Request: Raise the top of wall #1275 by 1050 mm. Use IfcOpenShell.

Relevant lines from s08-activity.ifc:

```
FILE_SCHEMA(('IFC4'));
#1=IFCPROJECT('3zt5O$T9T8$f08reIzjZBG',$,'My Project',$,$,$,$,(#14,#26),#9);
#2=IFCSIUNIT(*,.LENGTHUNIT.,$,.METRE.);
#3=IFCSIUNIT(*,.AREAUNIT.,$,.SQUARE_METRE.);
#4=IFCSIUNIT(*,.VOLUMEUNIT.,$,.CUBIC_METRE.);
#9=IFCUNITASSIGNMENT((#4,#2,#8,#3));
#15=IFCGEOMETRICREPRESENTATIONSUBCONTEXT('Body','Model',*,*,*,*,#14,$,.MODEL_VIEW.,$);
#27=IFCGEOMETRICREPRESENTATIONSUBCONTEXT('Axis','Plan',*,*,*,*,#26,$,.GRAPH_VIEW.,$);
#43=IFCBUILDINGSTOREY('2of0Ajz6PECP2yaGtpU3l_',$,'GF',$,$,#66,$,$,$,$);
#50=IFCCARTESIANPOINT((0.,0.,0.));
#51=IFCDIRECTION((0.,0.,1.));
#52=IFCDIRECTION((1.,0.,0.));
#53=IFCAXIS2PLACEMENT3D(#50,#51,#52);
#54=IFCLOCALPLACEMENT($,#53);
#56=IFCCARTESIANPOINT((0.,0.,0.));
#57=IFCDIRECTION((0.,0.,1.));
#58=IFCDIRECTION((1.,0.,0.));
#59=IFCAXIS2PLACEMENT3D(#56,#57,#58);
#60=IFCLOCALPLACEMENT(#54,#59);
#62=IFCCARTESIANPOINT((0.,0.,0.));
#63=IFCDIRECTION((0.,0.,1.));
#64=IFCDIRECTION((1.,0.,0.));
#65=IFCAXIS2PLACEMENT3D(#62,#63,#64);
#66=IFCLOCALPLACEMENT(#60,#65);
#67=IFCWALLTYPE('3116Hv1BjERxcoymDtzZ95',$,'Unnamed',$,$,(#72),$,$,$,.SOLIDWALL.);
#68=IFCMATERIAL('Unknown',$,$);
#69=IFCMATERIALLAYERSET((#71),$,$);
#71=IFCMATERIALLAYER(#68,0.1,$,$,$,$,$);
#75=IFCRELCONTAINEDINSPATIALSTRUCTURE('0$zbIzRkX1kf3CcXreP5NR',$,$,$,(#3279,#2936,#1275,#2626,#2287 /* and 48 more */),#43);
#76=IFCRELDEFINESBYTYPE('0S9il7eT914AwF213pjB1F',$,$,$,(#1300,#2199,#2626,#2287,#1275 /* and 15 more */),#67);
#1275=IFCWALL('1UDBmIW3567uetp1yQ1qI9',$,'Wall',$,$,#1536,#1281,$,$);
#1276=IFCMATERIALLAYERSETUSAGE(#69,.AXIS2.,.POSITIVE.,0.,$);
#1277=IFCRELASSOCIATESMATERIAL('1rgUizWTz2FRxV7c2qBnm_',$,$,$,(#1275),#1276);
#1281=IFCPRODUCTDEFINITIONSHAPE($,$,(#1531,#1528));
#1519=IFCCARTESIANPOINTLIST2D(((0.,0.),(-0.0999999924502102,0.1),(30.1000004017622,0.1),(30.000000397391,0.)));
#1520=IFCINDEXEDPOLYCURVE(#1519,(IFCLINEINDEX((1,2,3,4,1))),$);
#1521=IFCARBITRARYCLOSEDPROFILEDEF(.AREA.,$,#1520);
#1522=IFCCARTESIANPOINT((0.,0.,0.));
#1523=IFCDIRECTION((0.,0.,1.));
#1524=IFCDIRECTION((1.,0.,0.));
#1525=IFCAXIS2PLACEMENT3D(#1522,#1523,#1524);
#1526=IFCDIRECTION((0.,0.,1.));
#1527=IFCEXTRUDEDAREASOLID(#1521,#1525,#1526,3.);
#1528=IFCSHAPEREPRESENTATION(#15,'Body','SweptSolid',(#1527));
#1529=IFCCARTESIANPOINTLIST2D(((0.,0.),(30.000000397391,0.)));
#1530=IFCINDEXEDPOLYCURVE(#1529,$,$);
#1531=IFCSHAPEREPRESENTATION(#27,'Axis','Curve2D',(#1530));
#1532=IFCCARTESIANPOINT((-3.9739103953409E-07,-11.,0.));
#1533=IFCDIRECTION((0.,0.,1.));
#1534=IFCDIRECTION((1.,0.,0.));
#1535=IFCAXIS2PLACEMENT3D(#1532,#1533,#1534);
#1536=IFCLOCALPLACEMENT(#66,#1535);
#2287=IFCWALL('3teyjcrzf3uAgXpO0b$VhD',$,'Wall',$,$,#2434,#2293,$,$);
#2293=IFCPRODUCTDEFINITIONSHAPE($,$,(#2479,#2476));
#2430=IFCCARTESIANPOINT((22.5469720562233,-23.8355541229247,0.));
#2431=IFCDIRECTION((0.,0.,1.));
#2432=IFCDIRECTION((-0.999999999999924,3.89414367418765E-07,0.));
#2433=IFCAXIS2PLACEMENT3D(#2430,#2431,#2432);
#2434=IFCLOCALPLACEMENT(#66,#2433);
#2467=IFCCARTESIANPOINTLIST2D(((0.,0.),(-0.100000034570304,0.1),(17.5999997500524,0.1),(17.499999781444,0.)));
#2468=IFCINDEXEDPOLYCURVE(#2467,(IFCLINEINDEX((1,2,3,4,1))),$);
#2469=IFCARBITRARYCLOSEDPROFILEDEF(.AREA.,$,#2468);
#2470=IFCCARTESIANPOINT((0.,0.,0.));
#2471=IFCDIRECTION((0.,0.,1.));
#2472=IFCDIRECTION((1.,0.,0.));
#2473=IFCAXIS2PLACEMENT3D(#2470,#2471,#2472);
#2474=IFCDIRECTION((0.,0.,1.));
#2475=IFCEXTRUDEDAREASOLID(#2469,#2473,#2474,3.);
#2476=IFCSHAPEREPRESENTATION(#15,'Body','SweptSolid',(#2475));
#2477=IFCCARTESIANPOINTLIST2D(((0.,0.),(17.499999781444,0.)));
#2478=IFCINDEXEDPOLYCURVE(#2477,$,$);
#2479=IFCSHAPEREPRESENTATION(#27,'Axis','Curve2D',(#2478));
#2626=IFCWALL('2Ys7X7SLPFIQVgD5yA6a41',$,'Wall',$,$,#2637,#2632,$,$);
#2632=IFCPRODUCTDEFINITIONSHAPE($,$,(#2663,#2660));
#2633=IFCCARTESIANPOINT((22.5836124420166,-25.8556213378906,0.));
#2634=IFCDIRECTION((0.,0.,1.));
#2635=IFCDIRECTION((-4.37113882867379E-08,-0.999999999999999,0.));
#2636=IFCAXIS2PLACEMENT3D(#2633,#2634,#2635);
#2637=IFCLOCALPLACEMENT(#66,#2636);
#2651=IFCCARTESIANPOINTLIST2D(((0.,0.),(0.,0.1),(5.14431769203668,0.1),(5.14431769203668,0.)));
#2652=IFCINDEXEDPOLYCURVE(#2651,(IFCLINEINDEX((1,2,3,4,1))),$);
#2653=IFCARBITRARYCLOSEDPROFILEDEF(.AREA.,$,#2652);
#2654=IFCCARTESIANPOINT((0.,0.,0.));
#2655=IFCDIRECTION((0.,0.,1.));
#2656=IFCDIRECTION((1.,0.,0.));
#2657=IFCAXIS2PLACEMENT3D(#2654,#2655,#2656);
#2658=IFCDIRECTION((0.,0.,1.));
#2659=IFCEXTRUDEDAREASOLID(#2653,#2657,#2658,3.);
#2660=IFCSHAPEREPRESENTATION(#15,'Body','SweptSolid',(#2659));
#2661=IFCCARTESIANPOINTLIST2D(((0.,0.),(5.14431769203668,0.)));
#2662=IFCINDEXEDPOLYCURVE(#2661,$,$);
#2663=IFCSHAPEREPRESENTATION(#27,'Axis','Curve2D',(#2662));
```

```python
import ifcopenshell
import ifcopenshell.geom
import ifcopenshell.util.representation
import ifcopenshell.util.shape
import ifcopenshell.util.unit

model = ifcopenshell.open("s08-activity.ifc")
unit_scale = ifcopenshell.util.unit.calculate_unit_scale(model)
settings = ifcopenshell.geom.settings()


def volume(element):
    """Net volume in cubic metres, openings subtracted."""
    shape = ifcopenshell.geom.create_shape(settings, element)
    return ifcopenshell.util.shape.get_volume(shape.geometry)


wall = model.by_guid("1UDBmIW3567uetp1yQ1qI9")
before = volume(wall)

body = ifcopenshell.util.representation.get_representation(wall, "Model", "Body")
solid = body.Items[0]
old_height = solid.Depth
solid.Depth += 1.05 / unit_scale
after = volume(wall)

print(f"height {old_height:g} -> {solid.Depth:g}, volume {before:.3f} -> {after:.3f} m3")

model.write("s08-activity_v2.ifc")
```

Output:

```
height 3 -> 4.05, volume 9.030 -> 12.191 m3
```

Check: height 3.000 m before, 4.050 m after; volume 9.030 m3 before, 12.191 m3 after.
